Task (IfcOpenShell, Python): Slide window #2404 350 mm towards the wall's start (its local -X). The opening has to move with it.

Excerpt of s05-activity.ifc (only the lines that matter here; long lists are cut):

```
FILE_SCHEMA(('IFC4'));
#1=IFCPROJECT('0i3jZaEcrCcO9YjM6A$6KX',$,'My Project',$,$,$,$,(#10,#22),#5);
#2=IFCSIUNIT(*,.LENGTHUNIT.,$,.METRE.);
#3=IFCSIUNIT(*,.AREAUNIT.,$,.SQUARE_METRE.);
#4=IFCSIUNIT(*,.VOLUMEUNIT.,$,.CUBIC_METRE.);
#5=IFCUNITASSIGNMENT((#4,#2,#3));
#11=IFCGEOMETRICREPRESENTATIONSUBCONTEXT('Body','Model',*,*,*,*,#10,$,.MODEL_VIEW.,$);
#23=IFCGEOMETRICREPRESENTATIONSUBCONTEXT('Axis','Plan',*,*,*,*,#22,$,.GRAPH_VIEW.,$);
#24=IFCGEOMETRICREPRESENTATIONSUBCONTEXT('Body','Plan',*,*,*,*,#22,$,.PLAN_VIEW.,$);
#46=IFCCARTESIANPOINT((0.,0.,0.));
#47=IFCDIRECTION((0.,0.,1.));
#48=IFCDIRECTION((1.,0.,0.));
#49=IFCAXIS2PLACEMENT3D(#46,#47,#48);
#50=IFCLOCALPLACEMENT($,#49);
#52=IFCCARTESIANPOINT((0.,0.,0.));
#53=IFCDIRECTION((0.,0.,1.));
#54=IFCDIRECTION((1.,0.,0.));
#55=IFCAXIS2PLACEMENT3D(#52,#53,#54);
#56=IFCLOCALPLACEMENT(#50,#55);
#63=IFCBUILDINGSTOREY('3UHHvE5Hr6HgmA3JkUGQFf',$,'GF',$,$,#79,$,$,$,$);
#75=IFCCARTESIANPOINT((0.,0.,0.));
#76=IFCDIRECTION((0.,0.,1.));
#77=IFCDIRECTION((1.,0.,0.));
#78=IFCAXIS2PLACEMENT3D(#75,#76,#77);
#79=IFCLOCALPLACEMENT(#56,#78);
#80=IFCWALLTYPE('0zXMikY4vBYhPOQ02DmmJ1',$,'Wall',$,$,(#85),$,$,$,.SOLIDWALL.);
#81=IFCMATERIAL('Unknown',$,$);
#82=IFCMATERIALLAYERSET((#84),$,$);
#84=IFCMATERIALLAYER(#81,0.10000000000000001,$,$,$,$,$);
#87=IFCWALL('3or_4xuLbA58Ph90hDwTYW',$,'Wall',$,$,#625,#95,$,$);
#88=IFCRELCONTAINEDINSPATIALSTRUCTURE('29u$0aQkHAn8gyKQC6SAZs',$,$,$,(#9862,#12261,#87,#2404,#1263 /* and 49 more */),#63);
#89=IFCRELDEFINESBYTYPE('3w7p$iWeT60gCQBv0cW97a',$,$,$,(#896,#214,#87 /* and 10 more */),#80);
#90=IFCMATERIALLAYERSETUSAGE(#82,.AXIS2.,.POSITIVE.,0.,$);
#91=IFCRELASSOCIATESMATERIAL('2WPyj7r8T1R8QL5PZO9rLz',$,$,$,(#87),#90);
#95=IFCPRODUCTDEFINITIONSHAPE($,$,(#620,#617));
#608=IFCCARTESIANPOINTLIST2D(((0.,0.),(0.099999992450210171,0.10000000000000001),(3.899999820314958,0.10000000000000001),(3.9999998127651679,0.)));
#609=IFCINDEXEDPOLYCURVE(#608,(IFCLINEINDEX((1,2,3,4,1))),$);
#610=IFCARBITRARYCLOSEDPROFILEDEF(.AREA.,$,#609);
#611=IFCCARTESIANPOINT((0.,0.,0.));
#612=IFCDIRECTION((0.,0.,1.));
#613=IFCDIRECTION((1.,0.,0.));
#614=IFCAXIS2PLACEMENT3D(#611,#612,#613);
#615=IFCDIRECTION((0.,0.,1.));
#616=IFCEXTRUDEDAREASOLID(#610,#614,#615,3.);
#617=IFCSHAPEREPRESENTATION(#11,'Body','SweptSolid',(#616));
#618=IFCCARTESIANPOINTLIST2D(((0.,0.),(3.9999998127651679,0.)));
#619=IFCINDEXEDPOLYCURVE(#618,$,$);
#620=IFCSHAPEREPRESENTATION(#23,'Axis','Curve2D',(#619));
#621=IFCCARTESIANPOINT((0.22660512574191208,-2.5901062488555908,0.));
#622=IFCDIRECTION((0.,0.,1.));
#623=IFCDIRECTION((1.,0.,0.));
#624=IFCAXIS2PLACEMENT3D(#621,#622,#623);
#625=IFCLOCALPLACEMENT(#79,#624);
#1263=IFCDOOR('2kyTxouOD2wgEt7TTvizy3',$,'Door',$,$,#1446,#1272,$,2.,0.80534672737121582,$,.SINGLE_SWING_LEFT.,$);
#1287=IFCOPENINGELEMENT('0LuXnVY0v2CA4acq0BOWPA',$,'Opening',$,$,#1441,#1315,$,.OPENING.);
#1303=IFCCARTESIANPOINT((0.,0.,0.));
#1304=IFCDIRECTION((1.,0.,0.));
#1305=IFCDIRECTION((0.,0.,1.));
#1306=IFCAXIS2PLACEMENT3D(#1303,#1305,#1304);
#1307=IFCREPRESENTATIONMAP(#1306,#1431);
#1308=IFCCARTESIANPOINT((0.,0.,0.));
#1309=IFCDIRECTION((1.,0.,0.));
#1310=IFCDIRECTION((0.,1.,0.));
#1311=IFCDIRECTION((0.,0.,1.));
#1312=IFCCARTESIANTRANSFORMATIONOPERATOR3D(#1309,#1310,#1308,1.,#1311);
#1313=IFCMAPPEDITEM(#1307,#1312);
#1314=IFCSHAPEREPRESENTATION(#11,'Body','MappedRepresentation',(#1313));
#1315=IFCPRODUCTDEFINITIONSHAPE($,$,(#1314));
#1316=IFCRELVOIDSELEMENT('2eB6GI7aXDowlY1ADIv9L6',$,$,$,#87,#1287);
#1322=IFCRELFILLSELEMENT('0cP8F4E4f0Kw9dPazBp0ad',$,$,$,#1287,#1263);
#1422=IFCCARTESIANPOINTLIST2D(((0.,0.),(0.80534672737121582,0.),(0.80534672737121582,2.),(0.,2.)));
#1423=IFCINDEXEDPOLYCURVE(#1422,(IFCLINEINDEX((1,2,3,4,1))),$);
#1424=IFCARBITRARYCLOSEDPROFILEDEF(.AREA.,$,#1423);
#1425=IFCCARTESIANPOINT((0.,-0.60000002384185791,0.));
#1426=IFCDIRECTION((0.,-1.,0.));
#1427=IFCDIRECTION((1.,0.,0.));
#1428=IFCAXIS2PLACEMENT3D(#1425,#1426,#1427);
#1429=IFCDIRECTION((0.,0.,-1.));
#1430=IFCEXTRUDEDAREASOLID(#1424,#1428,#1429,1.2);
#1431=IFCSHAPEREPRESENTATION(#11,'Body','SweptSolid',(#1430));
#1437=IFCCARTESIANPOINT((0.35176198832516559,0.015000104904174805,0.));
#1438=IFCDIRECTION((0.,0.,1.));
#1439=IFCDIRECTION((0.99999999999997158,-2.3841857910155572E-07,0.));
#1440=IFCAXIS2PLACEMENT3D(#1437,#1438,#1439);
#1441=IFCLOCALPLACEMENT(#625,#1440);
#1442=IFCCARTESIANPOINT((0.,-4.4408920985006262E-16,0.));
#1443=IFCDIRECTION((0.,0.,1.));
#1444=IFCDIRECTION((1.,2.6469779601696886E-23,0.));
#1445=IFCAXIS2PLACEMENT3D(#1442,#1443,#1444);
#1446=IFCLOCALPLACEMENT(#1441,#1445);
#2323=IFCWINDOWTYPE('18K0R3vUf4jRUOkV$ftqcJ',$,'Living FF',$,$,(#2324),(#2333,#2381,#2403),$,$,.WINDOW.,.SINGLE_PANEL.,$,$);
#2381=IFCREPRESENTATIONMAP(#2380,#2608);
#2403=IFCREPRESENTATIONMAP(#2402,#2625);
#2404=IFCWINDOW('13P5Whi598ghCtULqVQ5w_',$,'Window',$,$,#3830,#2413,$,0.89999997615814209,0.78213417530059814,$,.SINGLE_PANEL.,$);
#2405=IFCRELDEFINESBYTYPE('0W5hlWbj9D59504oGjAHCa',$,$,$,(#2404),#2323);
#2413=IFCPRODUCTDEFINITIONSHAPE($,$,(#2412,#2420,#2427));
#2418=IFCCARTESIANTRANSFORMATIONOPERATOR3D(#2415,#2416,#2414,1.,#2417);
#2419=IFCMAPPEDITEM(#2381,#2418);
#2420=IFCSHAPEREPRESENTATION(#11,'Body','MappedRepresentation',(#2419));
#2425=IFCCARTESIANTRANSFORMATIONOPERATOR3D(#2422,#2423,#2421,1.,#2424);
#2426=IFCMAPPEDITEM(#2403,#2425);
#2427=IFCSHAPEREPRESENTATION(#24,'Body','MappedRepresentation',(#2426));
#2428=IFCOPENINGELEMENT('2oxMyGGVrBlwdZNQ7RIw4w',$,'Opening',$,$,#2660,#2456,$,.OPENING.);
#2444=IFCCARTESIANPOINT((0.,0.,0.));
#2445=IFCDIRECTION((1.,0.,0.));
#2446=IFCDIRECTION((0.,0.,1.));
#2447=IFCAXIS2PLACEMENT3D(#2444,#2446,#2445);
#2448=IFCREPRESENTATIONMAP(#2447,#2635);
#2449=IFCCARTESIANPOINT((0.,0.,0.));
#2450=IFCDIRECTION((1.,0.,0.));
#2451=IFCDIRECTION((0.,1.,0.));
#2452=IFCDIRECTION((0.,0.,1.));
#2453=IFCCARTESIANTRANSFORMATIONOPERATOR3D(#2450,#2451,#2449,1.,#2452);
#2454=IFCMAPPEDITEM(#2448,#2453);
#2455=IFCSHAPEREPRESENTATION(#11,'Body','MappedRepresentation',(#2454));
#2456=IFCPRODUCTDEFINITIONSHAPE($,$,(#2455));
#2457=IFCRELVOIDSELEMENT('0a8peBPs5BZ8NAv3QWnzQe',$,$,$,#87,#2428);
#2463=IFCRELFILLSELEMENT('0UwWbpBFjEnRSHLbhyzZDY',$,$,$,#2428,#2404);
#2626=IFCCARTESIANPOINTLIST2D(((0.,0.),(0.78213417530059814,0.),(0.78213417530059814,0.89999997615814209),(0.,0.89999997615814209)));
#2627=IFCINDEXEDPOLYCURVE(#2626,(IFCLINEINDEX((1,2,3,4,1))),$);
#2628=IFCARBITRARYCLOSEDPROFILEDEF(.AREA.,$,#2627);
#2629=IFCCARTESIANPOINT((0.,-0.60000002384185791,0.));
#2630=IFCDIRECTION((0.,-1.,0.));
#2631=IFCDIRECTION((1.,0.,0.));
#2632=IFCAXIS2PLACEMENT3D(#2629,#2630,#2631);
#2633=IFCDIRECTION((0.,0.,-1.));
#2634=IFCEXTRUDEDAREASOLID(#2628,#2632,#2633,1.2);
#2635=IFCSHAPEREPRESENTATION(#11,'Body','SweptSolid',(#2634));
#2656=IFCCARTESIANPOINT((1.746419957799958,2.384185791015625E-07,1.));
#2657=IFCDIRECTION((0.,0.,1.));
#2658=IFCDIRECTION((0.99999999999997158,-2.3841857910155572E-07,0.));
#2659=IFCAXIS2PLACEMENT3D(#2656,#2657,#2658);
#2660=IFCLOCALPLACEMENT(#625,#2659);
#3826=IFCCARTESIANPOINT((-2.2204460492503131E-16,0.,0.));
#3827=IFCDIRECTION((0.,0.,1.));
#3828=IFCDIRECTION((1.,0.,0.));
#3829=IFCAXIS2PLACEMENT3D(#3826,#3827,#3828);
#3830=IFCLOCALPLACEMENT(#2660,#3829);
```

```python
import ifcopenshell
import ifcopenshell.api.geometry
import ifcopenshell.util.placement

model = ifcopenshell.open("s05-activity.ifc")

window = model.by_id(2404)
opening = window.FillsVoids[0].RelatingOpeningElement
wall = opening.VoidsElements[0].RelatingBuildingElement

wall_matrix = ifcopenshell.util.placement.get_local_placement(wall.ObjectPlacement)
shift = wall_matrix[:3, 0] * -0.35
before = ifcopenshell.util.placement.get_local_placement(window.ObjectPlacement)[:3, 3].copy()

# The window is placed relative to its opening, so it follows when the opening moves.
matrix = ifcopenshell.util.placement.get_local_placement(opening.ObjectPlacement)
matrix[:3, 3] += shift
ifcopenshell.api.geometry.edit_object_placement(
    model, product=opening, matrix=matrix, is_si=False, should_transform_children=True
)

after = ifcopenshell.util.placement.get_local_placement(window.ObjectPlacement)[:3, 3]
print("window moved by", (after - before).round(3) + 0.0)

model.write("s05-activity_rev.ifc")
```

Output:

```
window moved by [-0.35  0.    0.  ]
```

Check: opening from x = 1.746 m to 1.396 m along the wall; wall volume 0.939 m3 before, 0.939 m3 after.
